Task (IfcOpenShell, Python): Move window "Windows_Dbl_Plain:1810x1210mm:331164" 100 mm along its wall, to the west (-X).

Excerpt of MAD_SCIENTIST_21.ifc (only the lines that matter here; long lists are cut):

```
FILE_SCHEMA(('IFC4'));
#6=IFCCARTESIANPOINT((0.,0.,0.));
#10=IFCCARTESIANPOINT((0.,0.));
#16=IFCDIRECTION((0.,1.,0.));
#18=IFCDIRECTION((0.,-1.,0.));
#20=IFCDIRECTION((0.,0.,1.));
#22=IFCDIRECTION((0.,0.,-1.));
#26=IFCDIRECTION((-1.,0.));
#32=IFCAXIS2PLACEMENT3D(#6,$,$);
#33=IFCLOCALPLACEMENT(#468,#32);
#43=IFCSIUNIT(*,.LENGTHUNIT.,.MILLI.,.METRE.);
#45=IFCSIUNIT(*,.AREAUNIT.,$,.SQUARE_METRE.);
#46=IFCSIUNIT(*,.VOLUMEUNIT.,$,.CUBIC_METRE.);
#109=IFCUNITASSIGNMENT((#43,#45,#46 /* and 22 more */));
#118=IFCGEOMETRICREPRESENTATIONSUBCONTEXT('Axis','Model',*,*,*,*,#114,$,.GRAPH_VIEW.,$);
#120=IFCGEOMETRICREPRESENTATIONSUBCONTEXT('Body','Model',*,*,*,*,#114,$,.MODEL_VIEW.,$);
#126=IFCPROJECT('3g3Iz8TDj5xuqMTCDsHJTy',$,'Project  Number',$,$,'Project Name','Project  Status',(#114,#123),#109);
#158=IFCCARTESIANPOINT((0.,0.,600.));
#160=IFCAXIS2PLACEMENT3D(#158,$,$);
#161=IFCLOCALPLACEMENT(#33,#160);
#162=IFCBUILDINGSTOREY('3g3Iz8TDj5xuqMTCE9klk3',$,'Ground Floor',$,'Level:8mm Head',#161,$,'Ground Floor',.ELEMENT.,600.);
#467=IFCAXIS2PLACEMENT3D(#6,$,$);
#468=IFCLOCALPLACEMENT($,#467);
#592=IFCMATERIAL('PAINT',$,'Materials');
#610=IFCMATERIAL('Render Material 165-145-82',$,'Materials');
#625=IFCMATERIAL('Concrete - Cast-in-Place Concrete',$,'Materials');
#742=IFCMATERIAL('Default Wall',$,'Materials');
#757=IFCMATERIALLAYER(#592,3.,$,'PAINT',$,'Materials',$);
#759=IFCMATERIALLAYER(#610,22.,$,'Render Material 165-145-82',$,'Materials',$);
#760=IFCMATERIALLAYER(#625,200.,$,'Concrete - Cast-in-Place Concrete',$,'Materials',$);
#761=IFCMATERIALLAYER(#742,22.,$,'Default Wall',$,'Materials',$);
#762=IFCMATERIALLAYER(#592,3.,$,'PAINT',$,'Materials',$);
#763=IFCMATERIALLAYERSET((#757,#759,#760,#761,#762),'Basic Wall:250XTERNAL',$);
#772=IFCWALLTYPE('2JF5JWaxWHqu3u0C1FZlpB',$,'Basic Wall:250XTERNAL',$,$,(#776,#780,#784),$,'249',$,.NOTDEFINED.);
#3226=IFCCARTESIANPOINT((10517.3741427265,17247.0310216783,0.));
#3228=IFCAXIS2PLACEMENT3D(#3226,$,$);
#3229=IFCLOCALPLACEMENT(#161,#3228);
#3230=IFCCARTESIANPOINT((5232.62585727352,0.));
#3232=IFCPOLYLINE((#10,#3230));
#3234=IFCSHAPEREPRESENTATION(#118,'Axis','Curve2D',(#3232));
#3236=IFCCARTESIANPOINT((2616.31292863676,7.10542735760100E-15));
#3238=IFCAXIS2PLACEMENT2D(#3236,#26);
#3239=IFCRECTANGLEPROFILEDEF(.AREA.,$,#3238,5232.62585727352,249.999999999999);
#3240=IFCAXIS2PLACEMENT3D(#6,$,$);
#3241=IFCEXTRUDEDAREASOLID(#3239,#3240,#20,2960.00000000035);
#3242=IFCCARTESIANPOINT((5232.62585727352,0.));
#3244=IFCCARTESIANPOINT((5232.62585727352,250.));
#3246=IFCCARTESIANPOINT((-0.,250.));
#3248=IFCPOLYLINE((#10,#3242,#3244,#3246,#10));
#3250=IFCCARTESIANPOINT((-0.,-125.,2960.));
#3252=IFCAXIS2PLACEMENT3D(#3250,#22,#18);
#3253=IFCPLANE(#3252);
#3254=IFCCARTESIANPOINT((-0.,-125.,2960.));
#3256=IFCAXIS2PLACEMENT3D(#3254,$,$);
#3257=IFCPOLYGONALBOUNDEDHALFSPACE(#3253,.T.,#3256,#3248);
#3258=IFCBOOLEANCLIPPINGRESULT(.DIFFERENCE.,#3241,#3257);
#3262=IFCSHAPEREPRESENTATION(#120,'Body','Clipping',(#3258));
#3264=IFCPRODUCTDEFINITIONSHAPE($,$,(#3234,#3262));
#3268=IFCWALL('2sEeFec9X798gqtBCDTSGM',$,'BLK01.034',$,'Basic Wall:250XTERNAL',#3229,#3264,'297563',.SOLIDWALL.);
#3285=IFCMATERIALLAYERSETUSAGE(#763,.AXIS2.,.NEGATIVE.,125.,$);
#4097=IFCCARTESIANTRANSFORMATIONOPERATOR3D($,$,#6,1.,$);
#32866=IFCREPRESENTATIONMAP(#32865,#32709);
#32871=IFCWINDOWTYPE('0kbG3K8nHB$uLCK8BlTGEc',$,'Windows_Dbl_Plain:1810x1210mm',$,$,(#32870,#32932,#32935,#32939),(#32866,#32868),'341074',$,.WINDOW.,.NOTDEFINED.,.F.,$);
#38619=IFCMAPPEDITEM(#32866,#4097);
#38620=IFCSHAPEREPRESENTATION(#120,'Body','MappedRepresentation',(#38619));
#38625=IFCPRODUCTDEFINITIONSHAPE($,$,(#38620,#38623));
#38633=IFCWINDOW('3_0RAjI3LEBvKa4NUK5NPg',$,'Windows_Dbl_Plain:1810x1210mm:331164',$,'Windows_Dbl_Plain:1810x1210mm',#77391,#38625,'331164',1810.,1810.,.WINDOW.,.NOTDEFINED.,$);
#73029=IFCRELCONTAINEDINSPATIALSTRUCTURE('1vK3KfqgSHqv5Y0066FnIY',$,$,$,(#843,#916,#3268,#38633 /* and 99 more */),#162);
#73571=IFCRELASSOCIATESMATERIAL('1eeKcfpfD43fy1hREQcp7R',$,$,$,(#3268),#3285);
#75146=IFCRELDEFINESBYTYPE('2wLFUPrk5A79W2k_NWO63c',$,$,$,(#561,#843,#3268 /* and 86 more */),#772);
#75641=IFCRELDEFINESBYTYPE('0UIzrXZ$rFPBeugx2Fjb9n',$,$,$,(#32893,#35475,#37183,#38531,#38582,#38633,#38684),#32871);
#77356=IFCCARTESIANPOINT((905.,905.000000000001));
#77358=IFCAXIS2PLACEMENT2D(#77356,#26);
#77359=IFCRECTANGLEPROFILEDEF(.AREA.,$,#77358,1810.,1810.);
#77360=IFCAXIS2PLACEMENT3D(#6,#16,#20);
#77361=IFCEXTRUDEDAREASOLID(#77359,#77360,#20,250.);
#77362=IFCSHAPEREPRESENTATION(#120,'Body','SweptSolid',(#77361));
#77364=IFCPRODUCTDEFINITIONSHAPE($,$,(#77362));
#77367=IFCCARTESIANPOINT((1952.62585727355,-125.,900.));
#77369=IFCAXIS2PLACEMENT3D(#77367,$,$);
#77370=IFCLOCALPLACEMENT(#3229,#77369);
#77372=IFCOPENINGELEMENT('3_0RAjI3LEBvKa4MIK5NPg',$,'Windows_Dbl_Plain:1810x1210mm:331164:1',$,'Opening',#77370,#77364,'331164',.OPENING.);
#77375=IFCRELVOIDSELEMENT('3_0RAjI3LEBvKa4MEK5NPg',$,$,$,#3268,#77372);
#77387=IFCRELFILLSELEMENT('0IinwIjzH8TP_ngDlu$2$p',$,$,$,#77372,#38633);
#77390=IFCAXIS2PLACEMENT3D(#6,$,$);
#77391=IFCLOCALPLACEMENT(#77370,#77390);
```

```python
import ifcopenshell
import ifcopenshell.api.geometry
import ifcopenshell.util.placement
import ifcopenshell.util.unit

model = ifcopenshell.open("MAD_SCIENTIST_21.ifc")
unit_scale = ifcopenshell.util.unit.calculate_unit_scale(model)

window = model.by_guid("3_0RAjI3LEBvKa4NUK5NPg")
opening = window.FillsVoids[0].RelatingOpeningElement
wall = opening.VoidsElements[0].RelatingBuildingElement

wall_matrix = ifcopenshell.util.placement.get_local_placement(wall.ObjectPlacement)
shift = wall_matrix[:3, 0] * -0.1 / unit_scale
before = ifcopenshell.util.placement.get_local_placement(window.ObjectPlacement)[:3, 3].copy()

# The window is placed relative to its opening, so it follows when the opening moves.
matrix = ifcopenshell.util.placement.get_local_placement(opening.ObjectPlacement)
matrix[:3, 3] += shift
ifcopenshell.api.geometry.edit_object_placement(
    model, product=opening, matrix=matrix, is_si=False, should_transform_children=True
)

after = ifcopenshell.util.placement.get_local_placement(window.ObjectPlacement)[:3, 3]
print("window moved by", (after - before).round(3) + 0.0)

model.write("MAD_SCIENTIST_21_edited.ifc")
```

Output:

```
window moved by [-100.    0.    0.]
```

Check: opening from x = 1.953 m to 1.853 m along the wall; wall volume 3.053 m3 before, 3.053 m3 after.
